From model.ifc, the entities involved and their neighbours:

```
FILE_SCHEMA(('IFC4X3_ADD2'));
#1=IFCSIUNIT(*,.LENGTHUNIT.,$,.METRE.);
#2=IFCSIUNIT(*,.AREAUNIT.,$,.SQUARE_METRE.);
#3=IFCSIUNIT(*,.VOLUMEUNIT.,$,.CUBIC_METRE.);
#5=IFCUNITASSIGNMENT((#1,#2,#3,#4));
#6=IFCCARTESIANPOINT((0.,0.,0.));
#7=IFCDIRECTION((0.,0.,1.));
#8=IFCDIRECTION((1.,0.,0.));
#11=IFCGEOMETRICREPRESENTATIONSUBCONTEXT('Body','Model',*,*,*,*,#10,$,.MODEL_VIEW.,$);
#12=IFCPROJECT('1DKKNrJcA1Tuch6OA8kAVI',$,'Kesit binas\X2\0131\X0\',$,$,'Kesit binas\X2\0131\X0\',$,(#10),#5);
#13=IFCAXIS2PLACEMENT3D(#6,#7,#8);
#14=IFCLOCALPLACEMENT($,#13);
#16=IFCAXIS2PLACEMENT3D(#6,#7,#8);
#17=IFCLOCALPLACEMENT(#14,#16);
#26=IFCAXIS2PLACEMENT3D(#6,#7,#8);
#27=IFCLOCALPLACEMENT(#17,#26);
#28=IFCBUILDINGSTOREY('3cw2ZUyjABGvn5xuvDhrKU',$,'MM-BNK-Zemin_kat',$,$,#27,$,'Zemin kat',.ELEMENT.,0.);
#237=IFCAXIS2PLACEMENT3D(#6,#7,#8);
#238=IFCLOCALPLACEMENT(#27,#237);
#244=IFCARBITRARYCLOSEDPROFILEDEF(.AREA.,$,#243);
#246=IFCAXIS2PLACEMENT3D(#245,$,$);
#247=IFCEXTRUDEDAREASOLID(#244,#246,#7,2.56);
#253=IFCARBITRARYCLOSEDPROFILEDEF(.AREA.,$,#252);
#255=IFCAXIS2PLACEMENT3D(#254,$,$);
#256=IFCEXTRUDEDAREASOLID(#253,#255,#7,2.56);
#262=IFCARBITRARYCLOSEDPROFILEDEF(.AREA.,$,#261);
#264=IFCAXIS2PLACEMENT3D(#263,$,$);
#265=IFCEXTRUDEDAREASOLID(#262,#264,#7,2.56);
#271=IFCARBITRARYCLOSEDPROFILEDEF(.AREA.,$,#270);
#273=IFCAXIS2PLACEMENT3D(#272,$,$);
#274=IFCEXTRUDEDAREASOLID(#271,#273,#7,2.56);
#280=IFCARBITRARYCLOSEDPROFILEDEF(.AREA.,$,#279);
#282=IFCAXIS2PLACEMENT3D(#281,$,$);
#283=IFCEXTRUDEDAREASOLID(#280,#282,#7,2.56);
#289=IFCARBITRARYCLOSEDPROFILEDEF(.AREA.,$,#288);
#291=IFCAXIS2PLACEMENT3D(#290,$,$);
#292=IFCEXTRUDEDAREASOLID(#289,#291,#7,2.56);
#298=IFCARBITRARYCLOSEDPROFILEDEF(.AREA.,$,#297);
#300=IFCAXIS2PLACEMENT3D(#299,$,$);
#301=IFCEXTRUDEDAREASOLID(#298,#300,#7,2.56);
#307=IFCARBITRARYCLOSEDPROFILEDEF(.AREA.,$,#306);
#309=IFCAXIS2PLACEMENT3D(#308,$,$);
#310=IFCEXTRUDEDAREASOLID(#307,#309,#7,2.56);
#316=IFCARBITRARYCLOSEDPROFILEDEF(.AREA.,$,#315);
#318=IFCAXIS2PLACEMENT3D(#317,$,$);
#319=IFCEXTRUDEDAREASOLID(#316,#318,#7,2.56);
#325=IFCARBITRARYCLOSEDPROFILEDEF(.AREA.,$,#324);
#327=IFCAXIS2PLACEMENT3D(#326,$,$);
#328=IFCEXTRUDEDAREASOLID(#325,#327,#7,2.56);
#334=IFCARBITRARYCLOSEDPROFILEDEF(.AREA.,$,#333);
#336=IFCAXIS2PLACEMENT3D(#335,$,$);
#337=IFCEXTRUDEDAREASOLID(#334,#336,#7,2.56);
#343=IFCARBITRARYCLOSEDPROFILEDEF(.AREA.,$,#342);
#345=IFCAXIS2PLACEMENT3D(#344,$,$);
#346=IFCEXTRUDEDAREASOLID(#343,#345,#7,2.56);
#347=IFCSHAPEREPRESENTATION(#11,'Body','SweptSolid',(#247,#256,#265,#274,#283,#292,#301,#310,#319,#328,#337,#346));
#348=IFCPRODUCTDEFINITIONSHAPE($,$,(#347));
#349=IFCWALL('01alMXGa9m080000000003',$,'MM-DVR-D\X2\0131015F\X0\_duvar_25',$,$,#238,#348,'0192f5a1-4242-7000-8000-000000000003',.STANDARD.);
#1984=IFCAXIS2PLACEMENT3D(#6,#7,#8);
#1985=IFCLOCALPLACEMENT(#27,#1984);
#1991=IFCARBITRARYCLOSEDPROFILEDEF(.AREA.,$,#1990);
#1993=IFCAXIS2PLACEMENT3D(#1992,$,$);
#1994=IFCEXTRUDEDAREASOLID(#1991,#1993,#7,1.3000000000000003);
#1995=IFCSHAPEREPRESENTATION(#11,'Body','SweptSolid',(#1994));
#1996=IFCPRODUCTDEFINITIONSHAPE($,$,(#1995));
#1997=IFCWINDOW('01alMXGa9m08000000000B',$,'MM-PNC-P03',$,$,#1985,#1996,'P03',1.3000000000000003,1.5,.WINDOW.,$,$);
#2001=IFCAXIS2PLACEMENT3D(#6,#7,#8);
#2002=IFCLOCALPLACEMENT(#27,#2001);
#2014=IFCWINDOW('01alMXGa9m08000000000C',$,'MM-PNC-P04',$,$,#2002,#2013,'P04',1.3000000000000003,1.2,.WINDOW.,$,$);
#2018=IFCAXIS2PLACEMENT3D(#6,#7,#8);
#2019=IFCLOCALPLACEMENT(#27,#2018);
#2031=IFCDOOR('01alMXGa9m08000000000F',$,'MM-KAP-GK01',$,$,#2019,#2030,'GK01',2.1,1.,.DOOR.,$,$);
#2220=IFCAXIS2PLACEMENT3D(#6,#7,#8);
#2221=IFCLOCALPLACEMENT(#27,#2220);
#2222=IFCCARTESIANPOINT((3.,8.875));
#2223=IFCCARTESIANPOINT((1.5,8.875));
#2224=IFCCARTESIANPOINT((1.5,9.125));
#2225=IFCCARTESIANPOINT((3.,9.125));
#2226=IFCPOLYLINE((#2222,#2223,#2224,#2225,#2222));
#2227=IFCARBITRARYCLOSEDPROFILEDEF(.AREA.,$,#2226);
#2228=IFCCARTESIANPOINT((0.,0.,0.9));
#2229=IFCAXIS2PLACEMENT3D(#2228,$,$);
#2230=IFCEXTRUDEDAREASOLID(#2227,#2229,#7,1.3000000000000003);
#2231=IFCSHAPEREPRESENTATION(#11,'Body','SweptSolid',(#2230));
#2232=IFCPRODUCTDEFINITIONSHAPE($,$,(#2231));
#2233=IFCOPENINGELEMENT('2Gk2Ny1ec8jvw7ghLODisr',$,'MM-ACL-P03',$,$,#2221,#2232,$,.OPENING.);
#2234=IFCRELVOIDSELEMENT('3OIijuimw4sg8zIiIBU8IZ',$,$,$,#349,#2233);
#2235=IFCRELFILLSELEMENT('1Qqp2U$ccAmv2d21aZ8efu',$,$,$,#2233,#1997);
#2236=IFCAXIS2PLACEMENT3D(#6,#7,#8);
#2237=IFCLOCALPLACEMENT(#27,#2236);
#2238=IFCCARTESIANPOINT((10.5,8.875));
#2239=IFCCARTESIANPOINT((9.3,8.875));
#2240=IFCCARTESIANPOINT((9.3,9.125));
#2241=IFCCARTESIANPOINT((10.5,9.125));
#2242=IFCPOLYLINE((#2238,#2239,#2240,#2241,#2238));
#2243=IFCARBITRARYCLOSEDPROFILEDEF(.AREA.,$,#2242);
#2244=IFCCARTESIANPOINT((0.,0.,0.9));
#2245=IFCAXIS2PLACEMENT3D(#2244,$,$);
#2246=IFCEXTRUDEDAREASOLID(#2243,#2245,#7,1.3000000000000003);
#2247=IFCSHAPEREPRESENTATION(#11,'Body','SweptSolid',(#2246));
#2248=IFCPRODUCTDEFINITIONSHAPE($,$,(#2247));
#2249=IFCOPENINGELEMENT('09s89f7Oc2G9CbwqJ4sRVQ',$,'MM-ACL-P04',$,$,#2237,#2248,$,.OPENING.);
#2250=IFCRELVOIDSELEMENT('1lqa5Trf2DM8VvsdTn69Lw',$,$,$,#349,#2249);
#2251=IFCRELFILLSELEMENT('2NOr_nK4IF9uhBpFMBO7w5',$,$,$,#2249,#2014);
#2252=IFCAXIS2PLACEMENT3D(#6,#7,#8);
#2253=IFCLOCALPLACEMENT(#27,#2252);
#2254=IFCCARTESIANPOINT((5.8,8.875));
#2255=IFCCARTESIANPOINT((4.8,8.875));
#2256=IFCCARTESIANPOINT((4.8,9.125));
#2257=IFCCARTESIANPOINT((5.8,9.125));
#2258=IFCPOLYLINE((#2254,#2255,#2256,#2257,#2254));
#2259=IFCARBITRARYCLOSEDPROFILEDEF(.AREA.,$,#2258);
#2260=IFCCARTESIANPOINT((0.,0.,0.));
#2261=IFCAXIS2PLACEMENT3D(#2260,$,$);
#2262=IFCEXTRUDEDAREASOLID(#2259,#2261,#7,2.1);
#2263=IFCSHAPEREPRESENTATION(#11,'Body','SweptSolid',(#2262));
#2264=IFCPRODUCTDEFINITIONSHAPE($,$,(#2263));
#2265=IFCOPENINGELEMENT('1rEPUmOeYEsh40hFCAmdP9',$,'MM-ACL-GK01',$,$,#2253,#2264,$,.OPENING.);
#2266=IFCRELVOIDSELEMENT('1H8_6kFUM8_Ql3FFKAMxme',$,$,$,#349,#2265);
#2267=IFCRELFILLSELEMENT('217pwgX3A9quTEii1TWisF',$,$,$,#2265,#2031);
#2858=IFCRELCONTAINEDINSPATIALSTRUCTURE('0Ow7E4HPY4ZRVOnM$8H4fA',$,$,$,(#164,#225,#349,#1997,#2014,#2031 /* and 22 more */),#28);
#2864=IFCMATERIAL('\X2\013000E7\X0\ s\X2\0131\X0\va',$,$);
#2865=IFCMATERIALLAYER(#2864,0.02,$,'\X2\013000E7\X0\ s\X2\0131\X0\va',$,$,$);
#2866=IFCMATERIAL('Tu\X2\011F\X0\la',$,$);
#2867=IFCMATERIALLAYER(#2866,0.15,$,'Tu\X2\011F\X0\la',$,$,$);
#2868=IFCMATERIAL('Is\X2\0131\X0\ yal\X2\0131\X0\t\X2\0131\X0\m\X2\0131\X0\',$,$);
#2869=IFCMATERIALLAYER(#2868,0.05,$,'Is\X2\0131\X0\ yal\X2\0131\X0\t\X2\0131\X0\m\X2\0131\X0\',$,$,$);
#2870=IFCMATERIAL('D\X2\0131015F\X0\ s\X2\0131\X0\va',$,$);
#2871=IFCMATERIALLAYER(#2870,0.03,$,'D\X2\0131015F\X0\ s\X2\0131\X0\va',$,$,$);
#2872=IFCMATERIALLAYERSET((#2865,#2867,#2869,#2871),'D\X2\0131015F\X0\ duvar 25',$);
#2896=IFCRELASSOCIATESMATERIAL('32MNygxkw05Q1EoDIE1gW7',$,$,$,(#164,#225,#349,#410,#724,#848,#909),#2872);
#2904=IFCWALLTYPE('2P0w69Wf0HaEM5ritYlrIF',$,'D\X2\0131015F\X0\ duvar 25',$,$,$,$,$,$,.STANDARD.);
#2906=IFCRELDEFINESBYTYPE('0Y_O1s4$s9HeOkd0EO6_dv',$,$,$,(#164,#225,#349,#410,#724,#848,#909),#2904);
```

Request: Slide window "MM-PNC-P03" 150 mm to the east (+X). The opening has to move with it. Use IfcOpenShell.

```python
import ifcopenshell
import ifcopenshell.api.geometry
import ifcopenshell.util.placement
import ifcopenshell.util.unit

model = ifcopenshell.open("model.ifc")
unit_scale = ifcopenshell.util.unit.calculate_unit_scale(model)

window = model.by_guid("01alMXGa9m08000000000B")
opening = window.FillsVoids[0].RelatingOpeningElement
wall = opening.VoidsElements[0].RelatingBuildingElement

wall_matrix = ifcopenshell.util.placement.get_local_placement(wall.ObjectPlacement)
shift = wall_matrix[:3, 0] * 0.15 / unit_scale
before = ifcopenshell.util.placement.get_local_placement(window.ObjectPlacement)[:3, 3].copy()

# The window is not placed relative to its opening, so move both.
for product in (opening, window):
    matrix = ifcopenshell.util.placement.get_local_placement(product.ObjectPlacement)
    matrix[:3, 3] += shift
    ifcopenshell.api.geometry.edit_object_placement(model, product=product, matrix=matrix, is_si=False)

after = ifcopenshell.util.placement.get_local_placement(window.ObjectPlacement)[:3, 3]
print("window moved by", (after - before).round(3) + 0.0)

model.write("model-out.ifc")
```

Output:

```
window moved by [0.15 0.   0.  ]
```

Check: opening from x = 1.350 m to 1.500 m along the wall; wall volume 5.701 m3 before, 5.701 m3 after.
